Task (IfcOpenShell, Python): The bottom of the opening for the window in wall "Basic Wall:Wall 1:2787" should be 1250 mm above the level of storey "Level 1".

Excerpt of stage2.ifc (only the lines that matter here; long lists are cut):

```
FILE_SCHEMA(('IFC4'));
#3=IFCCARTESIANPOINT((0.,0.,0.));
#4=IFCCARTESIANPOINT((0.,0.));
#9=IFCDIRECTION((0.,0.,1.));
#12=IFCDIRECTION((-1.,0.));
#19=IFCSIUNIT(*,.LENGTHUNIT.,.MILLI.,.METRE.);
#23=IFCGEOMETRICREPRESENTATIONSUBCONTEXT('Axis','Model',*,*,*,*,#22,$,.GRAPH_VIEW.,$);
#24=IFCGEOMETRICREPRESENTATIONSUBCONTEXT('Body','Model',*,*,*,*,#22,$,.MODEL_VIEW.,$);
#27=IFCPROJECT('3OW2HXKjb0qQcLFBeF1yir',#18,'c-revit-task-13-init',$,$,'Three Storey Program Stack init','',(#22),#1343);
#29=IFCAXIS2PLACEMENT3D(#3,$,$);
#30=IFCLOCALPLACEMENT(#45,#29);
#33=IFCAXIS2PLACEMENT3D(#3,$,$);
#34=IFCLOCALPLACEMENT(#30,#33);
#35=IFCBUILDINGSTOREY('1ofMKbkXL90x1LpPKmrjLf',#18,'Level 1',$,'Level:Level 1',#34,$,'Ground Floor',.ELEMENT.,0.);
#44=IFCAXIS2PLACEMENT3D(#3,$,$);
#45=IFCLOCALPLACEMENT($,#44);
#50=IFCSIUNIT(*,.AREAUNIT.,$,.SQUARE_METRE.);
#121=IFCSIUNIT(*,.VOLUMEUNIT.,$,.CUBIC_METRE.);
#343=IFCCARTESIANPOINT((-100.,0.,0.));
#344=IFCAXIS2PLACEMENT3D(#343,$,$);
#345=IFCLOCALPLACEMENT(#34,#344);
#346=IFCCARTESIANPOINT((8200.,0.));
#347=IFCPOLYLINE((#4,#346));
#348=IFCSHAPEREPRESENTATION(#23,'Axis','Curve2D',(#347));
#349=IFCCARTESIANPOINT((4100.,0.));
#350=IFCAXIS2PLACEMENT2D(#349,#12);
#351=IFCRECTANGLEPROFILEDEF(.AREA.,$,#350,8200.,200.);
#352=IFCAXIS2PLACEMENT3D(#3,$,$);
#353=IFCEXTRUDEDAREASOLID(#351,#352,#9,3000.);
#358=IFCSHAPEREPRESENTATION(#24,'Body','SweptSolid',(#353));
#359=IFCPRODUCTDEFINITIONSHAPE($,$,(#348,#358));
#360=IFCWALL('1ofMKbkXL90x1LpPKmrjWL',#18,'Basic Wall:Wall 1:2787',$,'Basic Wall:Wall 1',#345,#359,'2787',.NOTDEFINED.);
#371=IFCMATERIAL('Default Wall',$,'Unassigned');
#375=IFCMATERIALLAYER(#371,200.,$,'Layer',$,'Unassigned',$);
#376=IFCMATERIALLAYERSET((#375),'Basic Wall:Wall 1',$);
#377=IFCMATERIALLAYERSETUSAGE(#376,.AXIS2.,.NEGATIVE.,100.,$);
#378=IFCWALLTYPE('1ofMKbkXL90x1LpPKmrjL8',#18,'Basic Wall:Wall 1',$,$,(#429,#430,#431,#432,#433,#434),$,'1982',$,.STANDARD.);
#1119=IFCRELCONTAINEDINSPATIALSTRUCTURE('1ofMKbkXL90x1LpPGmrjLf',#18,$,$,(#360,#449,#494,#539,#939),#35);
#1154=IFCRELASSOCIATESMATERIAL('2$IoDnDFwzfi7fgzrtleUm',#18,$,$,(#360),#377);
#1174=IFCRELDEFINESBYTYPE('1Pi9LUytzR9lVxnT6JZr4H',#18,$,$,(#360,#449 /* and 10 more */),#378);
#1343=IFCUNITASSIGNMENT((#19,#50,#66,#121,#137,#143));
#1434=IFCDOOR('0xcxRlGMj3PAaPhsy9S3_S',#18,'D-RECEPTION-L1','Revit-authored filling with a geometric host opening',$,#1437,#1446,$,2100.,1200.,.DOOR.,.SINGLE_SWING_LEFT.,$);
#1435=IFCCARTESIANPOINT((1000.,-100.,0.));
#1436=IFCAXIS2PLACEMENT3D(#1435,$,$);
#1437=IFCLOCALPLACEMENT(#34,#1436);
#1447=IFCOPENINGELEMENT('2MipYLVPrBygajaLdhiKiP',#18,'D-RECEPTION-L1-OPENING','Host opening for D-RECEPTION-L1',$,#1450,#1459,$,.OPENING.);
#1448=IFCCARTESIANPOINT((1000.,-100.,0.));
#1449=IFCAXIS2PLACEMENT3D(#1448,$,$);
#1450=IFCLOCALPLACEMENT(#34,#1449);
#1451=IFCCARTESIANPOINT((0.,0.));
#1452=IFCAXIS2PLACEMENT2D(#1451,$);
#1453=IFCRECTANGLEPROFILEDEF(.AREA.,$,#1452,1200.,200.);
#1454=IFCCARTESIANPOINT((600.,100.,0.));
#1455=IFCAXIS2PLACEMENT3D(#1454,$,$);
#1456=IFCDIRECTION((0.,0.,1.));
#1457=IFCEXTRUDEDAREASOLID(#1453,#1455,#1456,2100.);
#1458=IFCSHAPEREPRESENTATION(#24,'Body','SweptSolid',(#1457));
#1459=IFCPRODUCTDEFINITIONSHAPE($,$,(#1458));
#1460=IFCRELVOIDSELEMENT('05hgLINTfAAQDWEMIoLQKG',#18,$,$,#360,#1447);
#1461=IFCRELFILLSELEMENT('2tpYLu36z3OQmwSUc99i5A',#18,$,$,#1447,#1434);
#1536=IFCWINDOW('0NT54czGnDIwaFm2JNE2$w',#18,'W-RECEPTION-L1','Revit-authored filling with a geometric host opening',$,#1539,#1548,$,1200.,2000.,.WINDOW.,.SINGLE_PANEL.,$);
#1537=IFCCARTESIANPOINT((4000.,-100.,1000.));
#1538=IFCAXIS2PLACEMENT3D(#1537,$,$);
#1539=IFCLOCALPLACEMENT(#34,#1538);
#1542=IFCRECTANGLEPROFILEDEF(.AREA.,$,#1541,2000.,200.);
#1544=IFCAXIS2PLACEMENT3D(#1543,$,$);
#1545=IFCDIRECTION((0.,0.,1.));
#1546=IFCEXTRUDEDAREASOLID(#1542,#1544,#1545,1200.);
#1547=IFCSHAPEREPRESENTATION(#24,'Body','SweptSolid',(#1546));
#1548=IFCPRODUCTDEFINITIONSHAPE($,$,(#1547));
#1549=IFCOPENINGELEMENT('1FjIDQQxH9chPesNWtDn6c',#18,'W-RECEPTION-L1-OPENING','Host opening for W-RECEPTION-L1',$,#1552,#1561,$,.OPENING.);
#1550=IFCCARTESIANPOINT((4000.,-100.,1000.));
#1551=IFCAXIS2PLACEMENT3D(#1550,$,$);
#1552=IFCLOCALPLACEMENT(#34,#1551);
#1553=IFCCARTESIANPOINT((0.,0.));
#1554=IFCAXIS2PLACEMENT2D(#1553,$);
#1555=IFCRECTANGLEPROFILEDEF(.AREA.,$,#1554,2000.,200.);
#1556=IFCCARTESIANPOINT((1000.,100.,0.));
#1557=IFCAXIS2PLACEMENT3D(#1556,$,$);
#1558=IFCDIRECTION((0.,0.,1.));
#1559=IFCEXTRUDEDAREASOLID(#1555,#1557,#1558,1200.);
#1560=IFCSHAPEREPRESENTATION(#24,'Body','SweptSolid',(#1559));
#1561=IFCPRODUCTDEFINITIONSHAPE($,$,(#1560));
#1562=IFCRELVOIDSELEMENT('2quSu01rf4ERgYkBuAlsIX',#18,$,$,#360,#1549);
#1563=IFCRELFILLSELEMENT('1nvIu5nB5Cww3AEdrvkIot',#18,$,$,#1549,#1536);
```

```python
import numpy as np
import ifcopenshell
import ifcopenshell.api.geometry
import ifcopenshell.geom
import ifcopenshell.util.element
import ifcopenshell.util.placement
import ifcopenshell.util.shape
import ifcopenshell.util.unit

model = ifcopenshell.open("stage2.ifc")
unit_scale = ifcopenshell.util.unit.calculate_unit_scale(model)

window = model.by_guid("0NT54czGnDIwaFm2JNE2$w")
opening = window.FillsVoids[0].RelatingOpeningElement
storey = ifcopenshell.util.element.get_container(window, ifc_class="IfcBuildingStorey")
level = ifcopenshell.util.placement.get_local_placement(storey.ObjectPlacement)[2, 3]

# The opening's origin need not be at the sill, so measure its lowest point.
shape = ifcopenshell.geom.create_shape(ifcopenshell.geom.settings(), opening)
bottom = ifcopenshell.util.shape.get_shape_bottom_elevation(shape, shape.geometry) / unit_scale
dz = level + 1.25 / unit_scale - bottom

shift = np.array([0.0, 0.0, dz])
# The window is not placed relative to its opening, so move both.
for product in (opening, window):
    matrix = ifcopenshell.util.placement.get_local_placement(product.ObjectPlacement)
    matrix[:3, 3] += shift
    ifcopenshell.api.geometry.edit_object_placement(model, product=product, matrix=matrix, is_si=False)

print(f"moved by {dz * unit_scale:+.3f} m")

model.write("stage2_v2.ifc")
```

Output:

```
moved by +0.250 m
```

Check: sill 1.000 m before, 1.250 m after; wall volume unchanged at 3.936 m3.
